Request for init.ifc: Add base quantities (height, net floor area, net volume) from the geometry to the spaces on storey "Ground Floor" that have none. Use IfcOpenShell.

First a look at what the model holds.

```python
import ifcopenshell
import ifcopenshell.util.element
import ifcopenshell.util.unit

model = ifcopenshell.open("init.ifc")
print(model.schema)
for unit_type in ("LENGTHUNIT", "AREAUNIT", "VOLUMEUNIT"):
    print(unit_type, ifcopenshell.util.unit.calculate_unit_scale(model, unit_type))
storey = next(s for s in model.by_type("IfcBuildingStorey") if s.Name == "Ground Floor")
spaces = [e for e in ifcopenshell.util.element.get_decomposition(storey) if e.is_a("IfcSpace")]
for e in sorted(spaces, key=lambda e: e.id()):
    print(e.id(), e.is_a(), e.Name, list(ifcopenshell.util.element.get_psets(e, qtos_only=True)), sep=" | ")
```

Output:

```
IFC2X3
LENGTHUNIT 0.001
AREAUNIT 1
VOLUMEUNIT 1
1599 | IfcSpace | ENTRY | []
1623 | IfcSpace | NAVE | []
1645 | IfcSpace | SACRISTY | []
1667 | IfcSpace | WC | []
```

```python
import ifcopenshell
import ifcopenshell.api.pset
import ifcopenshell.geom
import ifcopenshell.util.element
import ifcopenshell.util.shape
import ifcopenshell.util.unit

model = ifcopenshell.open("init.ifc")
unit_scale = ifcopenshell.util.unit.calculate_unit_scale(model)
area_scale = ifcopenshell.util.unit.calculate_unit_scale(model, "AREAUNIT")
volume_scale = ifcopenshell.util.unit.calculate_unit_scale(model, "VOLUMEUNIT")
settings = ifcopenshell.geom.settings()

storey = next(s for s in model.by_type("IfcBuildingStorey") if s.Name == "Ground Floor")
spaces = [e for e in ifcopenshell.util.element.get_decomposition(storey) if e.is_a("IfcSpace")]

for e in sorted(spaces, key=lambda e: e.id()):
    if ifcopenshell.util.element.get_psets(e, qtos_only=True, should_inherit=False):
        continue
    # Geometry comes back in metres, in the element's own axes.
    shape = ifcopenshell.geom.create_shape(settings, e)
    values = {
        "Height": ifcopenshell.util.shape.get_z(shape.geometry) / unit_scale,
        "NetFloorArea": ifcopenshell.util.shape.get_footprint_area(shape.geometry) / area_scale,
        "NetVolume": ifcopenshell.util.shape.get_volume(shape.geometry) / volume_scale,
    }
    qto = ifcopenshell.api.pset.add_qto(model, product=e, name="BaseQuantities")
    ifcopenshell.api.pset.edit_qto(model, qto=qto, properties=values)
    print(e.id(), {k: round(v, 3) for k, v in values.items()})

model.write("init_rev.ifc")
```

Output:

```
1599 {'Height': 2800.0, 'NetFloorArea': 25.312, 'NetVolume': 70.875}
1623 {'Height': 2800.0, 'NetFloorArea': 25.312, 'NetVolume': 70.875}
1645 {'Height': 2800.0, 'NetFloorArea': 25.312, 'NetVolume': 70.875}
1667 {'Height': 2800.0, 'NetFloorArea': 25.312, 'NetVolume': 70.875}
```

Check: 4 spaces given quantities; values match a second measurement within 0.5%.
